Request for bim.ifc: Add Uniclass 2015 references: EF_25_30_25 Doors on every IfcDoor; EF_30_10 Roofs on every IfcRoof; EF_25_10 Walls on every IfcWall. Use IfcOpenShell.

First a look at what the model holds.

```python
import ifcopenshell

model = ifcopenshell.open("bim.ifc")
print(model.schema)
print("classifications:", [c.Name for c in model.by_type("IfcClassification")])
for ifc_class in ("IfcDoor", "IfcRoof", "IfcStair", "IfcWall", "IfcWindow"):
    print(ifc_class, len(model.by_type(ifc_class)))
```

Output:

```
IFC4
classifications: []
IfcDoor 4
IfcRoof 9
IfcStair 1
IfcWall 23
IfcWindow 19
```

```python
import ifcopenshell
import ifcopenshell.api.classification

model = ifcopenshell.open("bim.ifc")

system = ifcopenshell.api.classification.add_classification(model, classification="Uniclass 2015")

codes = {
    "IfcDoor": ("EF_25_30_25", "Doors"),
    "IfcRoof": ("EF_30_10", "Roofs"),
    "IfcWall": ("EF_25_10", "Walls"),
}
for ifc_class, (code, name) in codes.items():
    products = model.by_type(ifc_class)
    ifcopenshell.api.classification.add_reference(
        model, products=products, classification=system, identification=code, name=name
    )
    print(code, len(products))

model.write("bim_rev.ifc")
```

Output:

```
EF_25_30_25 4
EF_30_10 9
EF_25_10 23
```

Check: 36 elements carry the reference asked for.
